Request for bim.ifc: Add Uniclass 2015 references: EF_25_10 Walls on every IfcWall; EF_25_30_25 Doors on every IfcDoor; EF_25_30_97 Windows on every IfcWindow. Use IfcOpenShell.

First a look at what the model holds.

```python
import ifcopenshell

model = ifcopenshell.open("bim.ifc")
print(model.schema)
print("classifications:", [c.Name for c in model.by_type("IfcClassification")])
for ifc_class in ("IfcDoor", "IfcRoof", "IfcStair", "IfcWall", "IfcWindow"):
    print(ifc_class, len(model.by_type(ifc_class)))
```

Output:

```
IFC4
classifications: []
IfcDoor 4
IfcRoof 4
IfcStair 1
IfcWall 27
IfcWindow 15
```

```python
import ifcopenshell
import ifcopenshell.api.classification

model = ifcopenshell.open("bim.ifc")

system = ifcopenshell.api.classification.add_classification(model, classification="Uniclass 2015")

codes = {
    "IfcWall": ("EF_25_10", "Walls"),
    "IfcDoor": ("EF_25_30_25", "Doors"),
    "IfcWindow": ("EF_25_30_97", "Windows"),
}
for ifc_class, (code, name) in codes.items():
    products = model.by_type(ifc_class)
    ifcopenshell.api.classification.add_reference(
        model, products=products, classification=system, identification=code, name=name
    )
    print(code, len(products))

model.write("bim_v2.ifc")
```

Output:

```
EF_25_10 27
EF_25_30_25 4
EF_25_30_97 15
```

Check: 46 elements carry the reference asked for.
